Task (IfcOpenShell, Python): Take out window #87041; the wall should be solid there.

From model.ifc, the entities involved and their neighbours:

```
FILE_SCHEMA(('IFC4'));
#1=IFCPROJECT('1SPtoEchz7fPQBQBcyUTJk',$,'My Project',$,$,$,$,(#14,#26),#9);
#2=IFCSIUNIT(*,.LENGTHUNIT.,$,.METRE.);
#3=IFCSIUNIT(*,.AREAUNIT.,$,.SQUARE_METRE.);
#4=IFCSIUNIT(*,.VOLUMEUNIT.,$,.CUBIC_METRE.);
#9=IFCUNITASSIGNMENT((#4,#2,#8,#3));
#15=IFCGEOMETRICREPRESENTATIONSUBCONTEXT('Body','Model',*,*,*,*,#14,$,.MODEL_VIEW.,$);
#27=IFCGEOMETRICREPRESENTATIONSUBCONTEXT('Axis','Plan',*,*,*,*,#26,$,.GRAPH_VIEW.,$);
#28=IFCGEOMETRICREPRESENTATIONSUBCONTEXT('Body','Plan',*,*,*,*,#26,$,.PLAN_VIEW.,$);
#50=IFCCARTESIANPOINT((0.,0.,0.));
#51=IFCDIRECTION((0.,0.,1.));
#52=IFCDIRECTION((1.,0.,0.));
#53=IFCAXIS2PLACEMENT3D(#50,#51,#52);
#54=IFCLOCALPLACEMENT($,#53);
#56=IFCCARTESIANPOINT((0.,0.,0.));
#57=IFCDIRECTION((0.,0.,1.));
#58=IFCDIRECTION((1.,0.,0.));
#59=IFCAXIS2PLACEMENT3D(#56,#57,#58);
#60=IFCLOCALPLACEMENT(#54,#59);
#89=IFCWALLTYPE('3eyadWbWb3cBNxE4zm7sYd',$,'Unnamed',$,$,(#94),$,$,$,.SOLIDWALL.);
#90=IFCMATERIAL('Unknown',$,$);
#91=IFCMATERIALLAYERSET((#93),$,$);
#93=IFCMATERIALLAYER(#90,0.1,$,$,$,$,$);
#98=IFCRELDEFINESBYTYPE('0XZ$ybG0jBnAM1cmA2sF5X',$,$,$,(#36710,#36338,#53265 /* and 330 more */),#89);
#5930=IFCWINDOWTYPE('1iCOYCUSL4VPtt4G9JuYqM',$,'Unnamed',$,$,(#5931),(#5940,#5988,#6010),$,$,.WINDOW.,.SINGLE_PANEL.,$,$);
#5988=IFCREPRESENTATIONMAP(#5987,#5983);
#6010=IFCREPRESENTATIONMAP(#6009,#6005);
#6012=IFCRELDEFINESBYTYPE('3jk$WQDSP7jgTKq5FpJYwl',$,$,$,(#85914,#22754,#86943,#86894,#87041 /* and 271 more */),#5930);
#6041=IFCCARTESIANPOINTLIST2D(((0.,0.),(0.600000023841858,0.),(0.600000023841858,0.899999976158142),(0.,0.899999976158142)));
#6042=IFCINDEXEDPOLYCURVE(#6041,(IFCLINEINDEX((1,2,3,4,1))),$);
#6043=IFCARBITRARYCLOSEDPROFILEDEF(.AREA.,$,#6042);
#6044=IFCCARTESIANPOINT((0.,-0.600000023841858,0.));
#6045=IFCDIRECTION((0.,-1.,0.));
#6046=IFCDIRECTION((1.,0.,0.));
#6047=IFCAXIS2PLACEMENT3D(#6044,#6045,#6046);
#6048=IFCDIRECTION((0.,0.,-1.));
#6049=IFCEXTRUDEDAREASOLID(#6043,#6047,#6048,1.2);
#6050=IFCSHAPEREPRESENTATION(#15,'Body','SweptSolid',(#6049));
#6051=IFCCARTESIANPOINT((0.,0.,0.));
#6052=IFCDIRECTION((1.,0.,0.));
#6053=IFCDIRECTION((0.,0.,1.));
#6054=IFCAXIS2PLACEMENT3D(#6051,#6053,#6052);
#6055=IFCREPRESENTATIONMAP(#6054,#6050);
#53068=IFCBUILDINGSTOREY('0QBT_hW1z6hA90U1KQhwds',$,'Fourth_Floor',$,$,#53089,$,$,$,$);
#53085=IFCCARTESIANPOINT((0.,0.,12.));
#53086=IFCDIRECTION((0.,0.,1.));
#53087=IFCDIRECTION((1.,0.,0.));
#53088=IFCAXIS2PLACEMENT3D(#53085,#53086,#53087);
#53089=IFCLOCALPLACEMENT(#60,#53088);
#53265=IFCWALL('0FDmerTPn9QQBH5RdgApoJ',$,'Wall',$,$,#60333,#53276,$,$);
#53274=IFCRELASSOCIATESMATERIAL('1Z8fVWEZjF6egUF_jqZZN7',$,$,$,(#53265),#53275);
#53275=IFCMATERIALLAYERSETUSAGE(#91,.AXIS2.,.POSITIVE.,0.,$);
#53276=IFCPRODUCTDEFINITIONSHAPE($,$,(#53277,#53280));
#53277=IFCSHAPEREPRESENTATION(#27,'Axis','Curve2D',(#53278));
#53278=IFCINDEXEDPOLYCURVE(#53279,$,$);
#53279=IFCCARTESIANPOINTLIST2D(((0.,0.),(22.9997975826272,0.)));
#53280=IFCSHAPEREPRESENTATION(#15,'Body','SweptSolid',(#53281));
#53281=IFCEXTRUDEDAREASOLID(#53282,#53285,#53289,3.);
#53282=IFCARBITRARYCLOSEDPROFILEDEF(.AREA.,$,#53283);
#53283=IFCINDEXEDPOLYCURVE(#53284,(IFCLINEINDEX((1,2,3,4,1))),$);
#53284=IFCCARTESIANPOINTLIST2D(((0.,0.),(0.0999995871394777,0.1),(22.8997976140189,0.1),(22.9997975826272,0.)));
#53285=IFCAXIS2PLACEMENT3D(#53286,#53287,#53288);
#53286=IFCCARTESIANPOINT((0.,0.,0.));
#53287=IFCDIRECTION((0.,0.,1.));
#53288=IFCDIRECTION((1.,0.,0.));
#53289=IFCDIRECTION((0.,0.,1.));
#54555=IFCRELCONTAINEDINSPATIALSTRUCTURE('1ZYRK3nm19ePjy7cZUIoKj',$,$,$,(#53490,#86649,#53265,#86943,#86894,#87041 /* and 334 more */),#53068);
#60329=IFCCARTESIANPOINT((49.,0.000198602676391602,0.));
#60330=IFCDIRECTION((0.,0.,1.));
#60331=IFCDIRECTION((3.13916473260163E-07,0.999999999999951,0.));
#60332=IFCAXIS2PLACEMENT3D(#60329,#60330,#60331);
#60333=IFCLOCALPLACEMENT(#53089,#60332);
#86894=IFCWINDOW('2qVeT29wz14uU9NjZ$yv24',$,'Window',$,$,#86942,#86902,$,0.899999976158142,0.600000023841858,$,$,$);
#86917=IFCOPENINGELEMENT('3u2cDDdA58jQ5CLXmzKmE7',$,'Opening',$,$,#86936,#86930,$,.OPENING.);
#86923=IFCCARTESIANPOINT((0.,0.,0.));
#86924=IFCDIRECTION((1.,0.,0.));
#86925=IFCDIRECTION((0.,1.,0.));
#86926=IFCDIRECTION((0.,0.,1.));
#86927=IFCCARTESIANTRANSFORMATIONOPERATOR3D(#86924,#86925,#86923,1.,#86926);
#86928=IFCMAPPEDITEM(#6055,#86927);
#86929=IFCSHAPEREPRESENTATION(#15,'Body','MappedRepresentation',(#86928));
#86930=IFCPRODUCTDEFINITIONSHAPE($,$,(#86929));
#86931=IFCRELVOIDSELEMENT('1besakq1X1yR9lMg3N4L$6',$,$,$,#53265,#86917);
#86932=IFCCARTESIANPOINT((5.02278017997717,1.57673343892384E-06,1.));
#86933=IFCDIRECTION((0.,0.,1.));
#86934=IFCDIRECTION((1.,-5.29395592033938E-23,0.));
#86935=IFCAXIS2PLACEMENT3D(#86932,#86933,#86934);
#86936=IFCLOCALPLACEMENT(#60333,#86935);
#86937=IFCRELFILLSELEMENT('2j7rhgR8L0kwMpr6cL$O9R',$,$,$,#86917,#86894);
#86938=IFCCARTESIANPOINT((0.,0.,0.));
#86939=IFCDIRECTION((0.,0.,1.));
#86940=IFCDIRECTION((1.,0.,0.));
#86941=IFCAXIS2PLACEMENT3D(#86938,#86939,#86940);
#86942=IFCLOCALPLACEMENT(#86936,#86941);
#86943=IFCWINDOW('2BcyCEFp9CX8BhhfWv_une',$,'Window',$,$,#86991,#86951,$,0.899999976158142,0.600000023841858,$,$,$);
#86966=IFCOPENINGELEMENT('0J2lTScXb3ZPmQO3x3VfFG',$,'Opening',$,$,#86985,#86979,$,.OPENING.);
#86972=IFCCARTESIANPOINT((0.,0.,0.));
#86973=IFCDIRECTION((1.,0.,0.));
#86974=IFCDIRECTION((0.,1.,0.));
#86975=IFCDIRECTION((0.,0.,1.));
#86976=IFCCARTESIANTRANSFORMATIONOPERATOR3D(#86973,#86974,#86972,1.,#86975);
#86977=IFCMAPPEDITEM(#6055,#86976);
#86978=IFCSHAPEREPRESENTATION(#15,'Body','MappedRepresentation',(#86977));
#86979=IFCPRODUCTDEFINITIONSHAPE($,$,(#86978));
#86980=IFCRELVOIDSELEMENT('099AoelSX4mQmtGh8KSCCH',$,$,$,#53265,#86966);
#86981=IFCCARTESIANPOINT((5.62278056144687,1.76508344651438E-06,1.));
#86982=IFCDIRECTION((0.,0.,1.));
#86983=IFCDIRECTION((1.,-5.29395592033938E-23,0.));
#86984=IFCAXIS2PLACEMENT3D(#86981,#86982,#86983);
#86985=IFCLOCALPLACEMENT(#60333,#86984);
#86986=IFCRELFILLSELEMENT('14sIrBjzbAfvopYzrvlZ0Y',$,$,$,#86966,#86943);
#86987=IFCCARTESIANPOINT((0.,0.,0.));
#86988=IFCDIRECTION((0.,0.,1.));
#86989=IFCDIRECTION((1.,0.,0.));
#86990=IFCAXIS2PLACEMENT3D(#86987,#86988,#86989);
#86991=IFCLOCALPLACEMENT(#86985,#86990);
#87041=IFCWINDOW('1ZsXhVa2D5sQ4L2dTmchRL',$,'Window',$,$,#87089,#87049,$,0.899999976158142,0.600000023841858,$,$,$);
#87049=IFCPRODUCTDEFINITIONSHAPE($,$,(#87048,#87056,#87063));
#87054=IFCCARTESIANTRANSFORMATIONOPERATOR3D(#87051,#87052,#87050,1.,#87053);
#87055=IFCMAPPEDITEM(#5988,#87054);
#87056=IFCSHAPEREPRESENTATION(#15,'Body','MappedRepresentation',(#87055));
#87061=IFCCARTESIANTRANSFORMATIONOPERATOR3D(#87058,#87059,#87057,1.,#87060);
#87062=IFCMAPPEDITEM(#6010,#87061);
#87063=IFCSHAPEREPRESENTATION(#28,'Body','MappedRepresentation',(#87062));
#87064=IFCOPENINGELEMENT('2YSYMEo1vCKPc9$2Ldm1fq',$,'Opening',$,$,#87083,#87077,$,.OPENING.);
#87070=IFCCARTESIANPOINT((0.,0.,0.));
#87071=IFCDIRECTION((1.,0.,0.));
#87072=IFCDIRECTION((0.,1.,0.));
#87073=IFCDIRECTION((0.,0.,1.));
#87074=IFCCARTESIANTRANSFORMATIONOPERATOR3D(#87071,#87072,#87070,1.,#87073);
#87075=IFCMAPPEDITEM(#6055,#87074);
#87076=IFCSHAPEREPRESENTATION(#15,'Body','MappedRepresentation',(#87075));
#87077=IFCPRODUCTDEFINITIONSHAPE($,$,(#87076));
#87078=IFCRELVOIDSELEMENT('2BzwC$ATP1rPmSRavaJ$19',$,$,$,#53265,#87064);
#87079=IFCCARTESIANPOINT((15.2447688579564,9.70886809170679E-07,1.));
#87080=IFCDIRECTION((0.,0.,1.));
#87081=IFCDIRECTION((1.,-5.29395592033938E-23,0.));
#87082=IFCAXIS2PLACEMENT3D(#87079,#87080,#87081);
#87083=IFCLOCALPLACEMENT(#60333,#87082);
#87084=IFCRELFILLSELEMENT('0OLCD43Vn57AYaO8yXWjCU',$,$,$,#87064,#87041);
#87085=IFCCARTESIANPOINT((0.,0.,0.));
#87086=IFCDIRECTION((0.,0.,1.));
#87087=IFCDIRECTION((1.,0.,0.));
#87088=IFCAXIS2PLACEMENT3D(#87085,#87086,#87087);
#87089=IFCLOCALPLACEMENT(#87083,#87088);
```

```python
import ifcopenshell
import ifcopenshell.api.feature
import ifcopenshell.api.root
import ifcopenshell.geom
import ifcopenshell.util.shape

model = ifcopenshell.open("model.ifc")
settings = ifcopenshell.geom.settings()


def volume(element):
    """Net volume in cubic metres, openings subtracted."""
    shape = ifcopenshell.geom.create_shape(settings, element)
    return ifcopenshell.util.shape.get_volume(shape.geometry)


window = model.by_id(87041)
opening = window.FillsVoids[0].RelatingOpeningElement
wall = opening.VoidsElements[0].RelatingBuildingElement
before = volume(wall)

ifcopenshell.api.root.remove_product(model, product=window)
ifcopenshell.api.feature.remove_feature(model, feature=opening)

after = volume(wall)

print(f"wall volume {before:.3f} -> {after:.3f} m3")

model.write("model_edited.ifc")
```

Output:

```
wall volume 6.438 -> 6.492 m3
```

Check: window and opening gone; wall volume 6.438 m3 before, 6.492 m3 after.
